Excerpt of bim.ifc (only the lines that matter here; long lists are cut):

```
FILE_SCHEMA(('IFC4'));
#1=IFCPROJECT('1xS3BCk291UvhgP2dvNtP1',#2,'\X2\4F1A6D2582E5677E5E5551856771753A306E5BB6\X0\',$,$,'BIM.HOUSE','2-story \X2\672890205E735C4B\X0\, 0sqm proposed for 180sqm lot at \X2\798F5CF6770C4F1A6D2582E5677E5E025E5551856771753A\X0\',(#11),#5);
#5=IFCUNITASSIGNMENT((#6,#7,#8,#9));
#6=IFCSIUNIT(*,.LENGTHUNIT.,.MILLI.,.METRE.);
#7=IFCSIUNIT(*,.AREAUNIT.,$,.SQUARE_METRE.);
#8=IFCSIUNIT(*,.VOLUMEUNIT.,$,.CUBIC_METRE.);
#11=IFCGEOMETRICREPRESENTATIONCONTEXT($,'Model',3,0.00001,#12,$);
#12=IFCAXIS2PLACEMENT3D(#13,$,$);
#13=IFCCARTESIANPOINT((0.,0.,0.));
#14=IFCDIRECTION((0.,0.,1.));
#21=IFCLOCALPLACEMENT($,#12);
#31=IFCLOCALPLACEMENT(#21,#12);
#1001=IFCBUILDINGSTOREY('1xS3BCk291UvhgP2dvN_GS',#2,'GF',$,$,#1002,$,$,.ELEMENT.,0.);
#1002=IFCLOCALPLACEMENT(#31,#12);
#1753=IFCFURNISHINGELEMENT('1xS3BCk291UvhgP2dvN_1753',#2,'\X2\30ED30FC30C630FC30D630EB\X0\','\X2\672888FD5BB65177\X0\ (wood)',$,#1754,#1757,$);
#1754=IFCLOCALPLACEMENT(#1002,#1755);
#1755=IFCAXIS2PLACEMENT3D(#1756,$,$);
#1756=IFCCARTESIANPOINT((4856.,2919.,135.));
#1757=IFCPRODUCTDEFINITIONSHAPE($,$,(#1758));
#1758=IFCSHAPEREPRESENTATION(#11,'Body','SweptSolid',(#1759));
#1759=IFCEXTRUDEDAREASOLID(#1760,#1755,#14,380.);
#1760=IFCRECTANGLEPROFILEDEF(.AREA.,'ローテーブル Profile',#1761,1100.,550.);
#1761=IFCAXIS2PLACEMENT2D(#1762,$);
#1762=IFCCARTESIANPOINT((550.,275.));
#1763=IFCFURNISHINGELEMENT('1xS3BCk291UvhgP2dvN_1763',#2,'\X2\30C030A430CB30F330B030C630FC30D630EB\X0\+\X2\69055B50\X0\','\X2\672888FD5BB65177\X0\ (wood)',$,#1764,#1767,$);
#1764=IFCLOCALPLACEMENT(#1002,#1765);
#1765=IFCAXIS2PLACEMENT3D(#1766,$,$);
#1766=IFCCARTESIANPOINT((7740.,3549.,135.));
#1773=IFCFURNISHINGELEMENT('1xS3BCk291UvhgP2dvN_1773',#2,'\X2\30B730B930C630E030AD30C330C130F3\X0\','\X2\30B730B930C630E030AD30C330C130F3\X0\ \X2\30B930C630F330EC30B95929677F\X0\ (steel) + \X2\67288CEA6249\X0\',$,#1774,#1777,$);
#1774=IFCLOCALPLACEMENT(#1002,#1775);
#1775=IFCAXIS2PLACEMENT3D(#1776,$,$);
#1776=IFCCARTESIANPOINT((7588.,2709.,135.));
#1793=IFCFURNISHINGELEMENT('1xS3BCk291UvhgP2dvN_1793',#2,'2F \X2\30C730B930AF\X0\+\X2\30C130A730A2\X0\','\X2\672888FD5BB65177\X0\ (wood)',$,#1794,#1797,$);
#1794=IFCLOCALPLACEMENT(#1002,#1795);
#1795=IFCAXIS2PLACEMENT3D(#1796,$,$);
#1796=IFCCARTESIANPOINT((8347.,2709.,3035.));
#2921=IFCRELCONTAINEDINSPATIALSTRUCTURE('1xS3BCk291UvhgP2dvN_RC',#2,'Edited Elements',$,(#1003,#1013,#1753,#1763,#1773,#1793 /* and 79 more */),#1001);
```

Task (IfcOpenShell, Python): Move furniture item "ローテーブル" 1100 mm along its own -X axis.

```python
import ifcopenshell
import ifcopenshell.api.geometry
import ifcopenshell.util.placement
import ifcopenshell.util.unit

model = ifcopenshell.open("bim.ifc")
unit_scale = ifcopenshell.util.unit.calculate_unit_scale(model)

item = model.by_id(1753)
matrix = ifcopenshell.util.placement.get_local_placement(item.ObjectPlacement)
matrix[:3, 3] -= matrix[:3, 0] * 1.1 / unit_scale
ifcopenshell.api.geometry.edit_object_placement(model, product=item, matrix=matrix, is_si=False)

print(ifcopenshell.util.placement.get_local_placement(item.ObjectPlacement).round(3) + 0.0)

model.write("bim-out.ifc")
```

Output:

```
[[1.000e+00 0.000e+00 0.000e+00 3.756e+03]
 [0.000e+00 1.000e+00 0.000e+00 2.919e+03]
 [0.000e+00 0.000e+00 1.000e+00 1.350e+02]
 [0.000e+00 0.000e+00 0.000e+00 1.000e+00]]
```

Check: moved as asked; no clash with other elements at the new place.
